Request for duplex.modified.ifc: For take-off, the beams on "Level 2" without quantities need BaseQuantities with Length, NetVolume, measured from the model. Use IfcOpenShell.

First a look at what the model holds.

```python
import ifcopenshell
import ifcopenshell.util.element
import ifcopenshell.util.unit

model = ifcopenshell.open("duplex.modified.ifc")
print(model.schema)
for unit_type in ("LENGTHUNIT", "AREAUNIT", "VOLUMEUNIT"):
    print(unit_type, ifcopenshell.util.unit.calculate_unit_scale(model, unit_type))
storey = next(s for s in model.by_type("IfcBuildingStorey") if s.Name == "Level 2")
beams = [e for e in ifcopenshell.util.element.get_decomposition(storey) if e.is_a("IfcBeam")]
for e in sorted(beams, key=lambda e: e.id()):
    print(e.id(), e.is_a(), e.Name, list(ifcopenshell.util.element.get_psets(e, qtos_only=True)), sep=" | ")
```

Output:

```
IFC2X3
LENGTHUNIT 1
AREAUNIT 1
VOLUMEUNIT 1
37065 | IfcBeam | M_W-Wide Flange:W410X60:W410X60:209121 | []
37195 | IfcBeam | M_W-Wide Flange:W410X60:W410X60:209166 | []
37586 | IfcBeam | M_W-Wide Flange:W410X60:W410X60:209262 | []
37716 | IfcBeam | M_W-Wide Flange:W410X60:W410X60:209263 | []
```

```python
import ifcopenshell
import ifcopenshell.api.pset
import ifcopenshell.geom
import ifcopenshell.util.element
import ifcopenshell.util.shape
import ifcopenshell.util.unit

model = ifcopenshell.open("duplex.modified.ifc")
unit_scale = ifcopenshell.util.unit.calculate_unit_scale(model)
volume_scale = ifcopenshell.util.unit.calculate_unit_scale(model, "VOLUMEUNIT")
settings = ifcopenshell.geom.settings()

storey = next(s for s in model.by_type("IfcBuildingStorey") if s.Name == "Level 2")
beams = [e for e in ifcopenshell.util.element.get_decomposition(storey) if e.is_a("IfcBeam")]

for e in sorted(beams, key=lambda e: e.id()):
    if ifcopenshell.util.element.get_psets(e, qtos_only=True, should_inherit=False):
        continue
    # Geometry comes back in metres, in the element's own axes.
    shape = ifcopenshell.geom.create_shape(settings, e)
    values = {
        "Length": ifcopenshell.util.shape.get_max_xyz(shape.geometry) / unit_scale,
        "NetVolume": ifcopenshell.util.shape.get_volume(shape.geometry) / volume_scale,
    }
    qto = ifcopenshell.api.pset.add_qto(model, product=e, name="BaseQuantities")
    ifcopenshell.api.pset.edit_qto(model, qto=qto, properties=values)
    print(e.id(), {k: round(v, 3) for k, v in values.items()})

model.write("duplex.modified_v2.ifc")
```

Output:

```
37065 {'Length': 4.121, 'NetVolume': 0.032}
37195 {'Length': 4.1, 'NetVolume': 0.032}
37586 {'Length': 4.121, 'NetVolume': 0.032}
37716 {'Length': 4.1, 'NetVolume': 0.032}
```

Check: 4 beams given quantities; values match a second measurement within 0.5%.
